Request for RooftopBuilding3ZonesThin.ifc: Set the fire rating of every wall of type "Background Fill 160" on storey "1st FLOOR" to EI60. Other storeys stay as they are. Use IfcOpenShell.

First a look at what the model holds.

```python
import ifcopenshell
import ifcopenshell.util.element

model = ifcopenshell.open("RooftopBuilding3ZonesThin.ifc")
print(model.schema)
storey = next(s for s in model.by_type("IfcBuildingStorey") if s.Name == "1st FLOOR")
walls = [e for e in ifcopenshell.util.element.get_decomposition(storey) if e.is_a("IfcWall")]
seen = {}
for e in walls:
    element_type = ifcopenshell.util.element.get_type(e)
    key = (element_type.Name if element_type != e and element_type else None, ifcopenshell.util.element.get_pset(e, "Pset_WallCommon", "FireRating"))
    seen[key] = seen.get(key, 0) + 1
for (name, value), count in sorted(seen.items(), key=str):
    print(count, "x", name, "|", value)
```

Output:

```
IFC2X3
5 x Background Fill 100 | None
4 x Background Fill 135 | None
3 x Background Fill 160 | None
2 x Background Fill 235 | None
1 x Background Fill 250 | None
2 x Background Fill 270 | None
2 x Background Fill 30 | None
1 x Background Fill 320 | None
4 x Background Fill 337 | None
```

```python
import ifcopenshell
import ifcopenshell.api.pset
import ifcopenshell.util.element

model = ifcopenshell.open("RooftopBuilding3ZonesThin.ifc")

storey = next(s for s in model.by_type("IfcBuildingStorey") if s.Name == "1st FLOOR")
walls = [e for e in ifcopenshell.util.element.get_decomposition(storey) if e.is_a("IfcWall")]

count = 0
for e in walls:
    element_type = ifcopenshell.util.element.get_type(e)
    if element_type in (None, e) or element_type.Name != "Background Fill 160":
        continue
    # add_pset returns the element's existing set when there is one.
    pset = ifcopenshell.api.pset.add_pset(model, product=e, name="Pset_WallCommon")
    ifcopenshell.api.pset.edit_pset(model, pset=pset, properties={"FireRating": "EI60"})
    count += 1

print(count, "walls updated")

model.write("RooftopBuilding3ZonesThin_v2.ifc")
```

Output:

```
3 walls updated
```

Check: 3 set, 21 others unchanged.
